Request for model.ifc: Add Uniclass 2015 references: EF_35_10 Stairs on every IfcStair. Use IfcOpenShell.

First a look at what the model holds.

```python
import ifcopenshell

model = ifcopenshell.open("model.ifc")
print(model.schema)
print("classifications:", [c.Name for c in model.by_type("IfcClassification")])
for ifc_class in ("IfcDoor", "IfcRoof", "IfcStair", "IfcWall", "IfcWindow"):
    print(ifc_class, len(model.by_type(ifc_class)))
```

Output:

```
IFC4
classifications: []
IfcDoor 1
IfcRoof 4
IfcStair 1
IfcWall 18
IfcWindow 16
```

```python
import ifcopenshell
import ifcopenshell.api.classification

model = ifcopenshell.open("model.ifc")

system = ifcopenshell.api.classification.add_classification(model, classification="Uniclass 2015")

codes = {
    "IfcStair": ("EF_35_10", "Stairs"),
}
for ifc_class, (code, name) in codes.items():
    products = model.by_type(ifc_class)
    ifcopenshell.api.classification.add_reference(
        model, products=products, classification=system, identification=code, name=name
    )
    print(code, len(products))

model.write("model_updated.ifc")
```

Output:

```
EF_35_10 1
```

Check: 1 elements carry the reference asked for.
